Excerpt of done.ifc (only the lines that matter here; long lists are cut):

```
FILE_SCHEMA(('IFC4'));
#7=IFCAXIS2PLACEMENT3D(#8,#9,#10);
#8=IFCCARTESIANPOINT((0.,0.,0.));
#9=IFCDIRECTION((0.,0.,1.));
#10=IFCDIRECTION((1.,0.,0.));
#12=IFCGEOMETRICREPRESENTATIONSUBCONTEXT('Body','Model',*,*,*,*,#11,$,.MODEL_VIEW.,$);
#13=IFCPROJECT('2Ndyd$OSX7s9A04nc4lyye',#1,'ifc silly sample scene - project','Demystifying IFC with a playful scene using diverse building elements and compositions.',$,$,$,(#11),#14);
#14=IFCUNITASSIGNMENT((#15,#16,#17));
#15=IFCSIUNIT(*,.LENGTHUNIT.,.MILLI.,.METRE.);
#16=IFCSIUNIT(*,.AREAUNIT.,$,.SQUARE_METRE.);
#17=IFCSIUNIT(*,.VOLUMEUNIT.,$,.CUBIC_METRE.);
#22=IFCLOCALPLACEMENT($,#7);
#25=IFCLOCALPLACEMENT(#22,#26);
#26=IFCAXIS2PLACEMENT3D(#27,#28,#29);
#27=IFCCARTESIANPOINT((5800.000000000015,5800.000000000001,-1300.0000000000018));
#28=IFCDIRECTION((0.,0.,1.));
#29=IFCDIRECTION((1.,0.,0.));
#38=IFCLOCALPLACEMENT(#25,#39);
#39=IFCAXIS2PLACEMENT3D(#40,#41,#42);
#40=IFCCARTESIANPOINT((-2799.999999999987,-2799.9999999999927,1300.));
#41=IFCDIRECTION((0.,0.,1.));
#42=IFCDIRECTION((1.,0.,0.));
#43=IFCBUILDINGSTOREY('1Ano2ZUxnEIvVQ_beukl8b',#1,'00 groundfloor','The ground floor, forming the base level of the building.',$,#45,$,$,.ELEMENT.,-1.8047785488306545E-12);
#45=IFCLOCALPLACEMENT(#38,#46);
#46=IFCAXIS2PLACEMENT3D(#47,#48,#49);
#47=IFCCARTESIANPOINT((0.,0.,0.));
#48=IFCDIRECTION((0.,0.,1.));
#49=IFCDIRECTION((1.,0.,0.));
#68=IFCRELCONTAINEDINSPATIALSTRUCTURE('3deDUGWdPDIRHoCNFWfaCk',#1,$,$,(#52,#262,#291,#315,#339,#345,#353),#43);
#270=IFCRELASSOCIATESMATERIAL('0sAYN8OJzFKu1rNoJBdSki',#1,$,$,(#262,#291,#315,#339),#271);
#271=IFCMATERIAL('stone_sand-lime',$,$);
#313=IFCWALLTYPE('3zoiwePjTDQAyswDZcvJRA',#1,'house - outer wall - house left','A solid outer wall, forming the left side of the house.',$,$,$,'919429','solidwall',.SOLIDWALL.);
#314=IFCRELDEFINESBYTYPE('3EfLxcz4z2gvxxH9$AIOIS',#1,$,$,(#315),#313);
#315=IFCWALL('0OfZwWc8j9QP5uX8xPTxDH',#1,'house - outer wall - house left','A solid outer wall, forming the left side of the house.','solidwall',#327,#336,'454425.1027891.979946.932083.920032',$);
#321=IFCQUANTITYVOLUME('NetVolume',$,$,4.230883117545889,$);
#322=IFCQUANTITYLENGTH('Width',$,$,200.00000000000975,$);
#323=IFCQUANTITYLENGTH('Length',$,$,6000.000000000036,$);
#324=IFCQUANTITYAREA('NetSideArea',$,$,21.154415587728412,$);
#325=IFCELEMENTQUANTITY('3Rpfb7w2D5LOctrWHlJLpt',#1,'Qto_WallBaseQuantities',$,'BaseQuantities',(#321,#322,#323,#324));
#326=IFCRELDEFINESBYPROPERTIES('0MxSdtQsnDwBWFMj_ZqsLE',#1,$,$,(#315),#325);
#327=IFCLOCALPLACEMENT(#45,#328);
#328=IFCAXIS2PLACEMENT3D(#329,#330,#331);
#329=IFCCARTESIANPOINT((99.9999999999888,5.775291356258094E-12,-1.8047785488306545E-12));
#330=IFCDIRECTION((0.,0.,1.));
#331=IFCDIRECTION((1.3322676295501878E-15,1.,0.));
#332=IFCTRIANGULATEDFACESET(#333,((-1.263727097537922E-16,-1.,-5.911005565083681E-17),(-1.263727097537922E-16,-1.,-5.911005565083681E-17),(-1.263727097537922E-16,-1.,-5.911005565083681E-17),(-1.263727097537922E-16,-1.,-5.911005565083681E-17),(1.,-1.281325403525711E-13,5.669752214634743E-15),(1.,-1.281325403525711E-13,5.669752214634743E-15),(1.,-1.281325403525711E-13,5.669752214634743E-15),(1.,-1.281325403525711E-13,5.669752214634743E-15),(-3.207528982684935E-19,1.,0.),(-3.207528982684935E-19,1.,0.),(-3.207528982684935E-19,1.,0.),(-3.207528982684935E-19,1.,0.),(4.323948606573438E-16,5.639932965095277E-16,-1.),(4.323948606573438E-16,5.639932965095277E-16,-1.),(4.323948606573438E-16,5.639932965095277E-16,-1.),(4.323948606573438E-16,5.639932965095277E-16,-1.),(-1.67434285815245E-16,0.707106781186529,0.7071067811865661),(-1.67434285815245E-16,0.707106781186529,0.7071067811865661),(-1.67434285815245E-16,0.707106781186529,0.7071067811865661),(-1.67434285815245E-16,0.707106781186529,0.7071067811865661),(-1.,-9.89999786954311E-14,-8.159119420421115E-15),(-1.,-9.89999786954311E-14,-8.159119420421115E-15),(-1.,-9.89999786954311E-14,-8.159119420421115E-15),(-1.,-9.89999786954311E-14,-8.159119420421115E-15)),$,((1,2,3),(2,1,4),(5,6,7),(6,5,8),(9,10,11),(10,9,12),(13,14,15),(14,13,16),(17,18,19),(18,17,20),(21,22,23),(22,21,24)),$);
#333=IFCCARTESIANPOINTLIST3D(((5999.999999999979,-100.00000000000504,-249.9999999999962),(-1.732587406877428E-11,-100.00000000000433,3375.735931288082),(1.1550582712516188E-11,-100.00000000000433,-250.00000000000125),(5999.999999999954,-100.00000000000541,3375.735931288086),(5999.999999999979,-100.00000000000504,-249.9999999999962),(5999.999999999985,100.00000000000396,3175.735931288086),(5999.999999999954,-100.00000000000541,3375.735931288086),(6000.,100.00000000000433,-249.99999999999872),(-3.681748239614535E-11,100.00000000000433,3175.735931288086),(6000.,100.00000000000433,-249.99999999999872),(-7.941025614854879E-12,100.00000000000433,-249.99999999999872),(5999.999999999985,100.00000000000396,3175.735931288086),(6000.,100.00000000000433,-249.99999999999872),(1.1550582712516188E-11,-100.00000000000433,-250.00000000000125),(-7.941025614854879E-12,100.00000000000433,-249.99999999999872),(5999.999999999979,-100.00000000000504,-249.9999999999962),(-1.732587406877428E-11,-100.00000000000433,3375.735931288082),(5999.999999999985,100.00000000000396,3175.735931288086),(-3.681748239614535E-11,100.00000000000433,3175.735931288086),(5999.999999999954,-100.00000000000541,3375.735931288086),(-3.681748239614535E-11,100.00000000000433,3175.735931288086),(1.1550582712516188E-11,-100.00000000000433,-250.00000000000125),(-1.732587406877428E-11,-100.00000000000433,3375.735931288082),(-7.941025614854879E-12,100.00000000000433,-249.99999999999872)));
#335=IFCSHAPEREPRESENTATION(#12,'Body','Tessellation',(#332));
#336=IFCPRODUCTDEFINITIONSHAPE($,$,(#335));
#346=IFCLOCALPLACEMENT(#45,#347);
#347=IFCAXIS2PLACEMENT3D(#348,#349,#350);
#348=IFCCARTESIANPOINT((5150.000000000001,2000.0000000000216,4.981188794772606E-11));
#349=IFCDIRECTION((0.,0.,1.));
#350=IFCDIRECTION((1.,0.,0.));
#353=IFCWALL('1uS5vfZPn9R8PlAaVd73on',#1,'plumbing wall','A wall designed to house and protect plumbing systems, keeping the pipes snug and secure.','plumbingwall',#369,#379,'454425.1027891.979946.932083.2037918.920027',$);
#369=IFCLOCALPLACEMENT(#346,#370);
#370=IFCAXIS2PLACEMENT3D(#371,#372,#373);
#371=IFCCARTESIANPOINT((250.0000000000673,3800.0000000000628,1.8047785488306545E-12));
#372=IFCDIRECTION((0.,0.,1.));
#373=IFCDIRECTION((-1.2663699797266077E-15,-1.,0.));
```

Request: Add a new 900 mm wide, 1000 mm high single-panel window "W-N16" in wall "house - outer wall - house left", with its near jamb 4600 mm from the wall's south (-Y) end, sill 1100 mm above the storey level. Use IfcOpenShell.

```python
import numpy as np
import ifcopenshell
import ifcopenshell.api.feature
import ifcopenshell.api.geometry
import ifcopenshell.api.pset
import ifcopenshell.api.root
import ifcopenshell.api.spatial
import ifcopenshell.geom
import ifcopenshell.util.element
import ifcopenshell.util.placement
import ifcopenshell.util.representation
import ifcopenshell.util.shape
import ifcopenshell.util.unit

model = ifcopenshell.open("done.ifc")
unit_scale = ifcopenshell.util.unit.calculate_unit_scale(model)
area_scale = ifcopenshell.util.unit.calculate_unit_scale(model, "AREAUNIT")
volume_scale = ifcopenshell.util.unit.calculate_unit_scale(model, "VOLUMEUNIT")
settings = ifcopenshell.geom.settings()


def volume(element):
    """Net volume in cubic metres, openings subtracted."""
    shape = ifcopenshell.geom.create_shape(settings, element)
    return ifcopenshell.util.shape.get_volume(shape.geometry)


wall = model.by_id(315)
storey = ifcopenshell.util.element.get_container(wall, ifc_class="IfcBuildingStorey")
context = ifcopenshell.util.representation.get_context(model, "Model", "Body", "MODEL_VIEW")
before = volume(wall)

width, height, from_end, sill = 0.9, 1, 4.6, 1.1  # metres

# The wall runs along its own X axis, and the end named is its -X end.
wall_shape = ifcopenshell.geom.create_shape(settings, wall)
x, y, z = ifcopenshell.util.shape.get_vertices(wall_shape.geometry).T
start = x.min() + from_end
face, thickness = float(y.min()), float(y.max() - y.min())
wall_matrix = ifcopenshell.util.placement.get_local_placement(wall.ObjectPlacement)
level = ifcopenshell.util.placement.get_local_placement(storey.ObjectPlacement)[2, 3]


def in_wall(x, y):
    """Placement at x, y metres in the wall's axes, at sill height."""
    matrix = wall_matrix.copy()
    matrix[:, 3] = wall_matrix @ np.array([x / unit_scale, y / unit_scale, 0.0, 1.0])
    matrix[2, 3] = level + sill / unit_scale
    return matrix


# Opening: a box that overshoots both wall faces by 50 mm.
opening = ifcopenshell.api.root.create_entity(model, ifc_class="IfcOpeningElement", predefined_type="OPENING")
box = ifcopenshell.api.geometry.add_wall_representation(
    model, context=context, length=width, height=height, thickness=thickness + 0.1
)
ifcopenshell.api.geometry.assign_representation(model, product=opening, representation=box)
ifcopenshell.api.geometry.edit_object_placement(model, product=opening, matrix=in_wall(start, face - 0.05), is_si=False)
ifcopenshell.api.feature.add_feature(model, feature=opening, element=wall)

window = ifcopenshell.api.root.create_entity(model, ifc_class="IfcWindow", name="W-N16", predefined_type="WINDOW")
window.OverallWidth, window.OverallHeight = width / unit_scale, height / unit_scale
window.PartitioningType = "SINGLE_PANEL"
body = ifcopenshell.api.geometry.add_window_representation(
    model,
    context=context,
    overall_width=window.OverallWidth,
    overall_height=window.OverallHeight,
    partition_type="SINGLE_PANEL",
)
ifcopenshell.api.geometry.assign_representation(model, product=window, representation=body)
ifcopenshell.api.spatial.assign_container(model, products=[window], relating_structure=storey)
ifcopenshell.api.feature.add_filling(model, opening=opening, element=window)

# Centre the window in the wall's thickness.
ifcopenshell.api.geometry.edit_object_placement(model, product=window, matrix=in_wall(start, face), is_si=False)
window_shape = ifcopenshell.geom.create_shape(settings, window)
depth = ifcopenshell.util.shape.get_vertices(window_shape.geometry)[:, 1]
offset = face + thickness / 2 - (depth.min() + depth.max()) / 2
ifcopenshell.api.geometry.edit_object_placement(model, product=window, matrix=in_wall(start, offset), is_si=False)

after = volume(wall)

# Update the wall's stored quantities.
qto = model.by_id(ifcopenshell.util.element.get_pset(wall, "Qto_WallBaseQuantities", should_inherit=False)["id"])
ifcopenshell.api.pset.edit_qto(model, qto=qto, properties={
    "NetVolume": after / volume_scale,
    "NetSideArea": after / thickness / area_scale,
})

print(f"wall volume {before:.3f} -> {after:.3f} m3")

model.write("done_rev.ifc")
```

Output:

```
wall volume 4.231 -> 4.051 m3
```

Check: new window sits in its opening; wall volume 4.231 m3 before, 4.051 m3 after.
